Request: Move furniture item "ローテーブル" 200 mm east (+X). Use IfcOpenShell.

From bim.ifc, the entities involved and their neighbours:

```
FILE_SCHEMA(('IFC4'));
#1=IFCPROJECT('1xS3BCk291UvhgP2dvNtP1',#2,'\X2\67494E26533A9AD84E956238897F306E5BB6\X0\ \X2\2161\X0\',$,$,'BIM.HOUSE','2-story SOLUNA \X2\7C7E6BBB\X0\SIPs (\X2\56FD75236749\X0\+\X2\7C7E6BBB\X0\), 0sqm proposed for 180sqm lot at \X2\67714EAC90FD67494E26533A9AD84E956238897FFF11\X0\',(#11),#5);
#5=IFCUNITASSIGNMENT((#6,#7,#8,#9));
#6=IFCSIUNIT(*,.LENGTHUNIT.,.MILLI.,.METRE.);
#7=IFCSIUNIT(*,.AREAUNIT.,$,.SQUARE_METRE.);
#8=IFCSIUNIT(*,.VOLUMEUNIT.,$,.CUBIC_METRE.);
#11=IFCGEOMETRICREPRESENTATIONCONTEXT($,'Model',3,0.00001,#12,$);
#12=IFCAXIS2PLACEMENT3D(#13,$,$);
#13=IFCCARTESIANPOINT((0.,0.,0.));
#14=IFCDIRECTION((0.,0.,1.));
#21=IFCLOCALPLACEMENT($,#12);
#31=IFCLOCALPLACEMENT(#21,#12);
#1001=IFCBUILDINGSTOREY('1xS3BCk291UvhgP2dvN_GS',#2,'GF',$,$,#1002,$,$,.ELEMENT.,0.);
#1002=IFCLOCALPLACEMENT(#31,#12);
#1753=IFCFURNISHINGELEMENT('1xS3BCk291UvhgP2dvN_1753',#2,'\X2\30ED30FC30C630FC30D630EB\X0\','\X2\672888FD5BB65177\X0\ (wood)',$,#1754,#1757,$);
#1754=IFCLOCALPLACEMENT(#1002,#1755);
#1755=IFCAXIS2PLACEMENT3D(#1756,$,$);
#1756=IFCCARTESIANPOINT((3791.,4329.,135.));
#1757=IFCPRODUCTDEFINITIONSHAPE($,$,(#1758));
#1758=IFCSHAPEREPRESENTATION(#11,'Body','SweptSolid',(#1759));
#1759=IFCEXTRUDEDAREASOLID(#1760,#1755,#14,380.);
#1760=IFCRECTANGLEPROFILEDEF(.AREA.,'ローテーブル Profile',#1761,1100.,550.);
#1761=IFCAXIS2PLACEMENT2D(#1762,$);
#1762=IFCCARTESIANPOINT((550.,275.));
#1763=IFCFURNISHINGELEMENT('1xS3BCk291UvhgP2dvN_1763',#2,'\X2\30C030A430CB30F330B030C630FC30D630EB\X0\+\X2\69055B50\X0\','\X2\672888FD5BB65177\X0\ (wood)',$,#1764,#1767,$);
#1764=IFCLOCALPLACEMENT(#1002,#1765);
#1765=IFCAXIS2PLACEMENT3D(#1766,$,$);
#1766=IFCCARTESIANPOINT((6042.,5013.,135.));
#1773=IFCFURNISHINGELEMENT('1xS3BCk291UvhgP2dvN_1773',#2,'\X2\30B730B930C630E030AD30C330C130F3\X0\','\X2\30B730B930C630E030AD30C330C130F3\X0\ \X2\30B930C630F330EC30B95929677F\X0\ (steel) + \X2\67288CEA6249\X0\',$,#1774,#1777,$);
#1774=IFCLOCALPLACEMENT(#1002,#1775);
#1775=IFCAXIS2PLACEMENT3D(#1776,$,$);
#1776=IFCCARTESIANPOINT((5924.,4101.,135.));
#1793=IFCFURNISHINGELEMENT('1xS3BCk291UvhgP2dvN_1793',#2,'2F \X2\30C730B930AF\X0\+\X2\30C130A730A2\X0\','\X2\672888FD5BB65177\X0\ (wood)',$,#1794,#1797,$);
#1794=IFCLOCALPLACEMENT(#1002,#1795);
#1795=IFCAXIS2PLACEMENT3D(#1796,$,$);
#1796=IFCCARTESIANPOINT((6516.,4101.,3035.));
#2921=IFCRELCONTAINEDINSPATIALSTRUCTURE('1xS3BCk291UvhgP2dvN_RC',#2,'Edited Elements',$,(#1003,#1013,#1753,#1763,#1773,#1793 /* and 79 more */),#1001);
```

```python
import ifcopenshell
import ifcopenshell.api.geometry
import ifcopenshell.util.placement
import ifcopenshell.util.unit

model = ifcopenshell.open("bim.ifc")
unit_scale = ifcopenshell.util.unit.calculate_unit_scale(model)

item = model.by_guid("1xS3BCk291UvhgP2dvN_1753")
matrix = ifcopenshell.util.placement.get_local_placement(item.ObjectPlacement)
matrix[0, 3] += 0.2 / unit_scale
ifcopenshell.api.geometry.edit_object_placement(model, product=item, matrix=matrix, is_si=False)

print(ifcopenshell.util.placement.get_local_placement(item.ObjectPlacement).round(3) + 0.0)

model.write("bim_updated.ifc")
```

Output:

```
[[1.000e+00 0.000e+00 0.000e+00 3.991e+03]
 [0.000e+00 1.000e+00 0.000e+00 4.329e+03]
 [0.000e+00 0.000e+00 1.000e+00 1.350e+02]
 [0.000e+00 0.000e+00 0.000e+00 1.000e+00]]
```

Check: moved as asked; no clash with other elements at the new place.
